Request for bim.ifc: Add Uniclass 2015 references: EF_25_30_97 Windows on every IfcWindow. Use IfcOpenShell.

First a look at what the model holds.

```python
import ifcopenshell

model = ifcopenshell.open("bim.ifc")
print(model.schema)
print("classifications:", [c.Name for c in model.by_type("IfcClassification")])
for ifc_class in ("IfcDoor", "IfcRoof", "IfcStair", "IfcWall", "IfcWindow"):
    print(ifc_class, len(model.by_type(ifc_class)))
```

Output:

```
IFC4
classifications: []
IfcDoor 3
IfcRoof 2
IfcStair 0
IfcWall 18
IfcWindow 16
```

```python
import ifcopenshell
import ifcopenshell.api.classification

model = ifcopenshell.open("bim.ifc")

system = ifcopenshell.api.classification.add_classification(model, classification="Uniclass 2015")

codes = {
    "IfcWindow": ("EF_25_30_97", "Windows"),
}
for ifc_class, (code, name) in codes.items():
    products = model.by_type(ifc_class)
    ifcopenshell.api.classification.add_reference(
        model, products=products, classification=system, identification=code, name=name
    )
    print(code, len(products))

model.write("bim_edited.ifc")
```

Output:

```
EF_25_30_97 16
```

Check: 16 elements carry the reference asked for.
